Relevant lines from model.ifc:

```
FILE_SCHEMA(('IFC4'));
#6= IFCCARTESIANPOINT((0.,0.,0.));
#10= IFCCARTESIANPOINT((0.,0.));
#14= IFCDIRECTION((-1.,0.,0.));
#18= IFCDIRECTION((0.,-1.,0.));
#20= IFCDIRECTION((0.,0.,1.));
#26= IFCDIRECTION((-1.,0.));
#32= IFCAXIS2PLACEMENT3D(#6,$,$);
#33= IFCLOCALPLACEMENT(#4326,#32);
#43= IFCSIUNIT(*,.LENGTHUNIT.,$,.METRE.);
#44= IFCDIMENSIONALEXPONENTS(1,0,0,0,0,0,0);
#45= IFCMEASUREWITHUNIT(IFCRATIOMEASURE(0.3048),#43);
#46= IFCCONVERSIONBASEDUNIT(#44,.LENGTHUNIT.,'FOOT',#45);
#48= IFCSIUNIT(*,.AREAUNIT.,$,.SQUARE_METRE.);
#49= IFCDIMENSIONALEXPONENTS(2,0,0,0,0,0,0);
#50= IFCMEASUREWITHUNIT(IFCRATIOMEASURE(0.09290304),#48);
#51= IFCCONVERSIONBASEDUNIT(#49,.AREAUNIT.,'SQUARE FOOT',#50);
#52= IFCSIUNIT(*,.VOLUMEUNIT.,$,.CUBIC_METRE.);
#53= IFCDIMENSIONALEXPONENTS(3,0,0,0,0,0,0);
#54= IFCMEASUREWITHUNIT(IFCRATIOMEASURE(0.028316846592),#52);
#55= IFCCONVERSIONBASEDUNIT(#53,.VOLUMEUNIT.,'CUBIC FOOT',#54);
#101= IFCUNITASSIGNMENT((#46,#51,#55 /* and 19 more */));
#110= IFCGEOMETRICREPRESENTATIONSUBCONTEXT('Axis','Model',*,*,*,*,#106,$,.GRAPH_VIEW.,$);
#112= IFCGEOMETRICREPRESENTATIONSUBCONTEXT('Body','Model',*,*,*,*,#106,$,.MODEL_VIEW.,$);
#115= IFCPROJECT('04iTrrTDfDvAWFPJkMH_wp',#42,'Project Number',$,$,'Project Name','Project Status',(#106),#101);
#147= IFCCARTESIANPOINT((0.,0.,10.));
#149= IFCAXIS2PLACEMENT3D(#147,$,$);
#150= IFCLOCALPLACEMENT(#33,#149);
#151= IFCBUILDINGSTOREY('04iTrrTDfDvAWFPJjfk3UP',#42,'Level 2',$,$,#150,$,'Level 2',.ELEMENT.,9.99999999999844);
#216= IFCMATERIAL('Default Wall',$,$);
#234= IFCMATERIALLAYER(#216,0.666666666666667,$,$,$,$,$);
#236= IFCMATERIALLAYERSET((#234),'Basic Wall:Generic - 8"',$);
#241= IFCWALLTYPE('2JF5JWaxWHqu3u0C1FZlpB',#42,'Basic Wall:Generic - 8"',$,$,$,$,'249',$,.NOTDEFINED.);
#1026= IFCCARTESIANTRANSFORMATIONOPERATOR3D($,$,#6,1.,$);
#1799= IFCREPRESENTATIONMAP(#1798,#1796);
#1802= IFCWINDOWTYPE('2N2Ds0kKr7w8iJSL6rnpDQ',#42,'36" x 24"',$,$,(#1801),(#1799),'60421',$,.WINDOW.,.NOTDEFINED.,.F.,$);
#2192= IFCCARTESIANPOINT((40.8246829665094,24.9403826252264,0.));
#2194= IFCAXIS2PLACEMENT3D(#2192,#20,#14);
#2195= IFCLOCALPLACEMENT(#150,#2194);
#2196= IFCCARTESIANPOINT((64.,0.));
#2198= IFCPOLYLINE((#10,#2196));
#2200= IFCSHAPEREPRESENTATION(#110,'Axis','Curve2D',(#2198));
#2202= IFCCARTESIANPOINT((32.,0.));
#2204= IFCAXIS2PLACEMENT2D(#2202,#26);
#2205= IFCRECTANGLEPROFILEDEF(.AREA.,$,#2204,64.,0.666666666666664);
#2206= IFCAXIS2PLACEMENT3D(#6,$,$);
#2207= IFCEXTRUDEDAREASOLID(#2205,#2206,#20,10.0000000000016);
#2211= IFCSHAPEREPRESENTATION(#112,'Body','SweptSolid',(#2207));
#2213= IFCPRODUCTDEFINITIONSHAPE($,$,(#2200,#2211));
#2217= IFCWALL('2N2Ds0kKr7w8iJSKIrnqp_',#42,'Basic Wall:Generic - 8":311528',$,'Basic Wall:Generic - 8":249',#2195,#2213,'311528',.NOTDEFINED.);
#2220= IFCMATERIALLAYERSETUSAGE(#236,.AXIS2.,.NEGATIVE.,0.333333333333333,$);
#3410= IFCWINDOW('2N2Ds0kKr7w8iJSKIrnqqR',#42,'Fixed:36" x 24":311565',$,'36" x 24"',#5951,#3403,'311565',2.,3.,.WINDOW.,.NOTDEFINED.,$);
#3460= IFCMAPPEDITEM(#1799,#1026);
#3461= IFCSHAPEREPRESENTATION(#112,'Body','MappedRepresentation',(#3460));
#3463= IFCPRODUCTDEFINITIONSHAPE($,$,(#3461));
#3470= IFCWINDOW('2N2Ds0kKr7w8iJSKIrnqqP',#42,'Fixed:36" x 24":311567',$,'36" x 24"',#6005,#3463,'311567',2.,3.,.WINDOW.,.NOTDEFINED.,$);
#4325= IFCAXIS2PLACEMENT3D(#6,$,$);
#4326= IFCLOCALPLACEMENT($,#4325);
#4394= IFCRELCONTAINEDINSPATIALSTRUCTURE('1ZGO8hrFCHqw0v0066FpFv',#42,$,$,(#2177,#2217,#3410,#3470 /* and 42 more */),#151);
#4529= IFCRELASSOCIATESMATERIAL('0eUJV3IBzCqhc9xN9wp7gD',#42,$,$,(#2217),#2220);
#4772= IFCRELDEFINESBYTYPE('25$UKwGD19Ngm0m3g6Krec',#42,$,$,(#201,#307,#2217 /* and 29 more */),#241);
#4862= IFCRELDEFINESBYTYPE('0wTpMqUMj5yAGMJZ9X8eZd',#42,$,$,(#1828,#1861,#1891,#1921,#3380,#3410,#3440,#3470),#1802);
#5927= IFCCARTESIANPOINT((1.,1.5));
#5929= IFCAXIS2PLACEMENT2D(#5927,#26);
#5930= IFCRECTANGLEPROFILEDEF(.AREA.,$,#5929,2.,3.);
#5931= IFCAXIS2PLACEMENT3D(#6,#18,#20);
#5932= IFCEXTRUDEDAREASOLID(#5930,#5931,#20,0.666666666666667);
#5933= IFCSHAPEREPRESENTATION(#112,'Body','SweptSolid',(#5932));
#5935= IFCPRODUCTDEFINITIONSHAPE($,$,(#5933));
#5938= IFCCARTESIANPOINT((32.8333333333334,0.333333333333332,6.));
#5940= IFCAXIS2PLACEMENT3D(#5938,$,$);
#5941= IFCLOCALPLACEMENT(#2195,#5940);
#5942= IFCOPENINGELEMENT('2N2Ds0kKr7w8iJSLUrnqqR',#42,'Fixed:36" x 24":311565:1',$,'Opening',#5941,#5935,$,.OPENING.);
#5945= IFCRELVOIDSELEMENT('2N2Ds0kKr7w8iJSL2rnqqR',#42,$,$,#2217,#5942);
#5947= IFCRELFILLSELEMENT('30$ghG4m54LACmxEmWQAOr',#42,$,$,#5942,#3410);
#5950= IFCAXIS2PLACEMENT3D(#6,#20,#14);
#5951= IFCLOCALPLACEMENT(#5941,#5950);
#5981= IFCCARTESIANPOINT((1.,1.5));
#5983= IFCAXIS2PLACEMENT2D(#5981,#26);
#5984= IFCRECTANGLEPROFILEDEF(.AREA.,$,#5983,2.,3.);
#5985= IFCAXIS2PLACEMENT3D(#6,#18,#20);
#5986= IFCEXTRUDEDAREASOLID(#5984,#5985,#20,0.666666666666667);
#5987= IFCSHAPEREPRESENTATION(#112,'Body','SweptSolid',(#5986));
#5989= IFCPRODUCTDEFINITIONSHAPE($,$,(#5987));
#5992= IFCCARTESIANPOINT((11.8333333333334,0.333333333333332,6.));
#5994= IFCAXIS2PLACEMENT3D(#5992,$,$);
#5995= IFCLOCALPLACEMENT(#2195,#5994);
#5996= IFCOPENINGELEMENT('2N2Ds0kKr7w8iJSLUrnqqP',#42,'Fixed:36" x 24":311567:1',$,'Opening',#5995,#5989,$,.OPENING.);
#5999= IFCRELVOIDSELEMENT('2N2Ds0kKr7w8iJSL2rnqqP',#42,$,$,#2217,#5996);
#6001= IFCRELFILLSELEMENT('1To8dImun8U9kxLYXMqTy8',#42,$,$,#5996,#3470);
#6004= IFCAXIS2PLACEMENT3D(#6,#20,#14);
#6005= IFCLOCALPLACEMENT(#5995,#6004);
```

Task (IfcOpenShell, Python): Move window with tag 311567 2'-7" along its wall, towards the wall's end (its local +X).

```python
import ifcopenshell
import ifcopenshell.api.geometry
import ifcopenshell.util.placement
import ifcopenshell.util.unit

model = ifcopenshell.open("model.ifc")
unit_scale = ifcopenshell.util.unit.calculate_unit_scale(model)

window = model.by_guid("2N2Ds0kKr7w8iJSKIrnqqP")
opening = window.FillsVoids[0].RelatingOpeningElement
wall = opening.VoidsElements[0].RelatingBuildingElement

wall_matrix = ifcopenshell.util.placement.get_local_placement(wall.ObjectPlacement)
shift = wall_matrix[:3, 0] * 31 * 0.0254 / unit_scale
before = ifcopenshell.util.placement.get_local_placement(window.ObjectPlacement)[:3, 3].copy()

# The window is placed relative to its opening, so it follows when the opening moves.
matrix = ifcopenshell.util.placement.get_local_placement(opening.ObjectPlacement)
matrix[:3, 3] += shift
ifcopenshell.api.geometry.edit_object_placement(
    model, product=opening, matrix=matrix, is_si=False, should_transform_children=True
)

after = ifcopenshell.util.placement.get_local_placement(window.ObjectPlacement)[:3, 3]
print("window moved by", (after - before).round(3) + 0.0)

model.write("model_updated.ifc")
```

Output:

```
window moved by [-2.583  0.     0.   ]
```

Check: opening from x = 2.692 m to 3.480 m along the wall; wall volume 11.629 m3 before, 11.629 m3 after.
